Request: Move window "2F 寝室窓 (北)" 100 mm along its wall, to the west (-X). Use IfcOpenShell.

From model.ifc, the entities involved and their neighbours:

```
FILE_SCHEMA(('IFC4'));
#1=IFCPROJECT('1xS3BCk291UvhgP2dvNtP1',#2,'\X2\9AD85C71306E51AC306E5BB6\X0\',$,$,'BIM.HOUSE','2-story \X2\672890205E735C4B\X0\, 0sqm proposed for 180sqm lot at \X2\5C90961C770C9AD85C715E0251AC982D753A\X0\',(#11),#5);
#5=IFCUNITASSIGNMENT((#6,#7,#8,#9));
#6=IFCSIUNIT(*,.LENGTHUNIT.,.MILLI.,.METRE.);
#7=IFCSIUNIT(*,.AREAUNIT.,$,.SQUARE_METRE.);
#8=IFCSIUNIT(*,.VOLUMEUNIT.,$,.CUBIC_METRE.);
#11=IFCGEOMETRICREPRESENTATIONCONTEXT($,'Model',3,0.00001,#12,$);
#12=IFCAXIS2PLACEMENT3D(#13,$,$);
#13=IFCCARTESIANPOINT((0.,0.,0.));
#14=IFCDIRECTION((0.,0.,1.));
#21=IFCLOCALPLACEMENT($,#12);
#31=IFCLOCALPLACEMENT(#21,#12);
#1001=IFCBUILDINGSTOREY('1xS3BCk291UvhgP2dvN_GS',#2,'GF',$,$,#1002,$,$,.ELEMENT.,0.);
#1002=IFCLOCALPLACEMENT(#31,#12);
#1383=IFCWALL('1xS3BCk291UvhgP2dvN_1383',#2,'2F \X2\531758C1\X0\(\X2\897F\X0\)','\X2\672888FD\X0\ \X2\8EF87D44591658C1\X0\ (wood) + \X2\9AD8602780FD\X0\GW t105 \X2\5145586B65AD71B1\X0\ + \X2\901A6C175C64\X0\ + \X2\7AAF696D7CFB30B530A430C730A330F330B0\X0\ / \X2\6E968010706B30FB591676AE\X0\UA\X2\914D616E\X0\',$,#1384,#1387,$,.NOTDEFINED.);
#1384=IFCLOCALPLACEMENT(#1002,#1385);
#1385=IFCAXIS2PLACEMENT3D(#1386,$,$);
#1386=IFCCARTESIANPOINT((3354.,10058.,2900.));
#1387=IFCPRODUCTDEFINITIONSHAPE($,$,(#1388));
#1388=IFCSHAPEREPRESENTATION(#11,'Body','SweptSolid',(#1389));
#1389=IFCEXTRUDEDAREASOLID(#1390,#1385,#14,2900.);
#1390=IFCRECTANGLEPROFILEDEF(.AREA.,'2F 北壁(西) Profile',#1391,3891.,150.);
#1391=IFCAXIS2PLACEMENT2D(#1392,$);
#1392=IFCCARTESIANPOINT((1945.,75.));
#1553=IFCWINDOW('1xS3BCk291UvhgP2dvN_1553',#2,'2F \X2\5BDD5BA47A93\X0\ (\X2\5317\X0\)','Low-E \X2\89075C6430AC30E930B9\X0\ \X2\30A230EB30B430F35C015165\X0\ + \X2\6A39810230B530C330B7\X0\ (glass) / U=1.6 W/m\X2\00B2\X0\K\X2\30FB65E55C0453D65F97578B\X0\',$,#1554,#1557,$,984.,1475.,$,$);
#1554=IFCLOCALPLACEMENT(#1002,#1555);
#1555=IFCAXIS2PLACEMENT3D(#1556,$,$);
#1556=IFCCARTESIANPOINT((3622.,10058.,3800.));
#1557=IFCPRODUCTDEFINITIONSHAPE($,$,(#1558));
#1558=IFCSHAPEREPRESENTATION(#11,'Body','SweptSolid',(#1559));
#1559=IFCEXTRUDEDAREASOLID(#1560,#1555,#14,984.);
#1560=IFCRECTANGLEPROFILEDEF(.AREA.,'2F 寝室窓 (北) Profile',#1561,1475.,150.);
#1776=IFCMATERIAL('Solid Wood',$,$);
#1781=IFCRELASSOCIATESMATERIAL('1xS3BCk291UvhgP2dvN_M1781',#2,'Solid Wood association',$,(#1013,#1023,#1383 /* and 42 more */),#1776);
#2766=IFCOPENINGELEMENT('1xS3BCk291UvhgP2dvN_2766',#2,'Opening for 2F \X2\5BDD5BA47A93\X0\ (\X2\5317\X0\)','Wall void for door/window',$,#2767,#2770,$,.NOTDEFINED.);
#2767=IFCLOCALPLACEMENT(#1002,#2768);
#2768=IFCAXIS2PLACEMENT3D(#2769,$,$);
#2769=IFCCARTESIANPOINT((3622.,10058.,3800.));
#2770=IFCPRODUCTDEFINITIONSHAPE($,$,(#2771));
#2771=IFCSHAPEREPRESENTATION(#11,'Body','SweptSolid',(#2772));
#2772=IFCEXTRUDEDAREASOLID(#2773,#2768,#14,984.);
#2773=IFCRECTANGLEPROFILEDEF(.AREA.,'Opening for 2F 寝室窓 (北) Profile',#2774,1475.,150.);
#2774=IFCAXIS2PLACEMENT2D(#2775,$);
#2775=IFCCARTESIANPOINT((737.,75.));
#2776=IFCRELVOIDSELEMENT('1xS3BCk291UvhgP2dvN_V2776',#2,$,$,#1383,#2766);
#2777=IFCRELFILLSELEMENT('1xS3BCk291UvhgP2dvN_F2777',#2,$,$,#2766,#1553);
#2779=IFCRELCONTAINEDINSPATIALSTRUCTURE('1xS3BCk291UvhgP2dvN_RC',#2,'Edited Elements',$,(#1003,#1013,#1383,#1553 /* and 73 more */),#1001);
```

```python
import ifcopenshell
import ifcopenshell.api.geometry
import ifcopenshell.util.placement

model = ifcopenshell.open("model.ifc")

window = model.by_id(1553)
opening = window.FillsVoids[0].RelatingOpeningElement
wall = opening.VoidsElements[0].RelatingBuildingElement

wall_matrix = ifcopenshell.util.placement.get_local_placement(wall.ObjectPlacement)
shift = wall_matrix[:3, 0] * -100.0
before = ifcopenshell.util.placement.get_local_placement(window.ObjectPlacement)[:3, 3].copy()

# The window is not placed relative to its opening, so move both.
for product in (opening, window):
    matrix = ifcopenshell.util.placement.get_local_placement(product.ObjectPlacement)
    matrix[:3, 3] += shift
    ifcopenshell.api.geometry.edit_object_placement(model, product=product, matrix=matrix, is_si=False)

after = ifcopenshell.util.placement.get_local_placement(window.ObjectPlacement)[:3, 3]
print("window moved by", (after - before).round(3) + 0.0)

model.write("model-out.ifc")
```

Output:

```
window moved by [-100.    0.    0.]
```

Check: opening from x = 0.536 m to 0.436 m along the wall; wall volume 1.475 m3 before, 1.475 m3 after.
